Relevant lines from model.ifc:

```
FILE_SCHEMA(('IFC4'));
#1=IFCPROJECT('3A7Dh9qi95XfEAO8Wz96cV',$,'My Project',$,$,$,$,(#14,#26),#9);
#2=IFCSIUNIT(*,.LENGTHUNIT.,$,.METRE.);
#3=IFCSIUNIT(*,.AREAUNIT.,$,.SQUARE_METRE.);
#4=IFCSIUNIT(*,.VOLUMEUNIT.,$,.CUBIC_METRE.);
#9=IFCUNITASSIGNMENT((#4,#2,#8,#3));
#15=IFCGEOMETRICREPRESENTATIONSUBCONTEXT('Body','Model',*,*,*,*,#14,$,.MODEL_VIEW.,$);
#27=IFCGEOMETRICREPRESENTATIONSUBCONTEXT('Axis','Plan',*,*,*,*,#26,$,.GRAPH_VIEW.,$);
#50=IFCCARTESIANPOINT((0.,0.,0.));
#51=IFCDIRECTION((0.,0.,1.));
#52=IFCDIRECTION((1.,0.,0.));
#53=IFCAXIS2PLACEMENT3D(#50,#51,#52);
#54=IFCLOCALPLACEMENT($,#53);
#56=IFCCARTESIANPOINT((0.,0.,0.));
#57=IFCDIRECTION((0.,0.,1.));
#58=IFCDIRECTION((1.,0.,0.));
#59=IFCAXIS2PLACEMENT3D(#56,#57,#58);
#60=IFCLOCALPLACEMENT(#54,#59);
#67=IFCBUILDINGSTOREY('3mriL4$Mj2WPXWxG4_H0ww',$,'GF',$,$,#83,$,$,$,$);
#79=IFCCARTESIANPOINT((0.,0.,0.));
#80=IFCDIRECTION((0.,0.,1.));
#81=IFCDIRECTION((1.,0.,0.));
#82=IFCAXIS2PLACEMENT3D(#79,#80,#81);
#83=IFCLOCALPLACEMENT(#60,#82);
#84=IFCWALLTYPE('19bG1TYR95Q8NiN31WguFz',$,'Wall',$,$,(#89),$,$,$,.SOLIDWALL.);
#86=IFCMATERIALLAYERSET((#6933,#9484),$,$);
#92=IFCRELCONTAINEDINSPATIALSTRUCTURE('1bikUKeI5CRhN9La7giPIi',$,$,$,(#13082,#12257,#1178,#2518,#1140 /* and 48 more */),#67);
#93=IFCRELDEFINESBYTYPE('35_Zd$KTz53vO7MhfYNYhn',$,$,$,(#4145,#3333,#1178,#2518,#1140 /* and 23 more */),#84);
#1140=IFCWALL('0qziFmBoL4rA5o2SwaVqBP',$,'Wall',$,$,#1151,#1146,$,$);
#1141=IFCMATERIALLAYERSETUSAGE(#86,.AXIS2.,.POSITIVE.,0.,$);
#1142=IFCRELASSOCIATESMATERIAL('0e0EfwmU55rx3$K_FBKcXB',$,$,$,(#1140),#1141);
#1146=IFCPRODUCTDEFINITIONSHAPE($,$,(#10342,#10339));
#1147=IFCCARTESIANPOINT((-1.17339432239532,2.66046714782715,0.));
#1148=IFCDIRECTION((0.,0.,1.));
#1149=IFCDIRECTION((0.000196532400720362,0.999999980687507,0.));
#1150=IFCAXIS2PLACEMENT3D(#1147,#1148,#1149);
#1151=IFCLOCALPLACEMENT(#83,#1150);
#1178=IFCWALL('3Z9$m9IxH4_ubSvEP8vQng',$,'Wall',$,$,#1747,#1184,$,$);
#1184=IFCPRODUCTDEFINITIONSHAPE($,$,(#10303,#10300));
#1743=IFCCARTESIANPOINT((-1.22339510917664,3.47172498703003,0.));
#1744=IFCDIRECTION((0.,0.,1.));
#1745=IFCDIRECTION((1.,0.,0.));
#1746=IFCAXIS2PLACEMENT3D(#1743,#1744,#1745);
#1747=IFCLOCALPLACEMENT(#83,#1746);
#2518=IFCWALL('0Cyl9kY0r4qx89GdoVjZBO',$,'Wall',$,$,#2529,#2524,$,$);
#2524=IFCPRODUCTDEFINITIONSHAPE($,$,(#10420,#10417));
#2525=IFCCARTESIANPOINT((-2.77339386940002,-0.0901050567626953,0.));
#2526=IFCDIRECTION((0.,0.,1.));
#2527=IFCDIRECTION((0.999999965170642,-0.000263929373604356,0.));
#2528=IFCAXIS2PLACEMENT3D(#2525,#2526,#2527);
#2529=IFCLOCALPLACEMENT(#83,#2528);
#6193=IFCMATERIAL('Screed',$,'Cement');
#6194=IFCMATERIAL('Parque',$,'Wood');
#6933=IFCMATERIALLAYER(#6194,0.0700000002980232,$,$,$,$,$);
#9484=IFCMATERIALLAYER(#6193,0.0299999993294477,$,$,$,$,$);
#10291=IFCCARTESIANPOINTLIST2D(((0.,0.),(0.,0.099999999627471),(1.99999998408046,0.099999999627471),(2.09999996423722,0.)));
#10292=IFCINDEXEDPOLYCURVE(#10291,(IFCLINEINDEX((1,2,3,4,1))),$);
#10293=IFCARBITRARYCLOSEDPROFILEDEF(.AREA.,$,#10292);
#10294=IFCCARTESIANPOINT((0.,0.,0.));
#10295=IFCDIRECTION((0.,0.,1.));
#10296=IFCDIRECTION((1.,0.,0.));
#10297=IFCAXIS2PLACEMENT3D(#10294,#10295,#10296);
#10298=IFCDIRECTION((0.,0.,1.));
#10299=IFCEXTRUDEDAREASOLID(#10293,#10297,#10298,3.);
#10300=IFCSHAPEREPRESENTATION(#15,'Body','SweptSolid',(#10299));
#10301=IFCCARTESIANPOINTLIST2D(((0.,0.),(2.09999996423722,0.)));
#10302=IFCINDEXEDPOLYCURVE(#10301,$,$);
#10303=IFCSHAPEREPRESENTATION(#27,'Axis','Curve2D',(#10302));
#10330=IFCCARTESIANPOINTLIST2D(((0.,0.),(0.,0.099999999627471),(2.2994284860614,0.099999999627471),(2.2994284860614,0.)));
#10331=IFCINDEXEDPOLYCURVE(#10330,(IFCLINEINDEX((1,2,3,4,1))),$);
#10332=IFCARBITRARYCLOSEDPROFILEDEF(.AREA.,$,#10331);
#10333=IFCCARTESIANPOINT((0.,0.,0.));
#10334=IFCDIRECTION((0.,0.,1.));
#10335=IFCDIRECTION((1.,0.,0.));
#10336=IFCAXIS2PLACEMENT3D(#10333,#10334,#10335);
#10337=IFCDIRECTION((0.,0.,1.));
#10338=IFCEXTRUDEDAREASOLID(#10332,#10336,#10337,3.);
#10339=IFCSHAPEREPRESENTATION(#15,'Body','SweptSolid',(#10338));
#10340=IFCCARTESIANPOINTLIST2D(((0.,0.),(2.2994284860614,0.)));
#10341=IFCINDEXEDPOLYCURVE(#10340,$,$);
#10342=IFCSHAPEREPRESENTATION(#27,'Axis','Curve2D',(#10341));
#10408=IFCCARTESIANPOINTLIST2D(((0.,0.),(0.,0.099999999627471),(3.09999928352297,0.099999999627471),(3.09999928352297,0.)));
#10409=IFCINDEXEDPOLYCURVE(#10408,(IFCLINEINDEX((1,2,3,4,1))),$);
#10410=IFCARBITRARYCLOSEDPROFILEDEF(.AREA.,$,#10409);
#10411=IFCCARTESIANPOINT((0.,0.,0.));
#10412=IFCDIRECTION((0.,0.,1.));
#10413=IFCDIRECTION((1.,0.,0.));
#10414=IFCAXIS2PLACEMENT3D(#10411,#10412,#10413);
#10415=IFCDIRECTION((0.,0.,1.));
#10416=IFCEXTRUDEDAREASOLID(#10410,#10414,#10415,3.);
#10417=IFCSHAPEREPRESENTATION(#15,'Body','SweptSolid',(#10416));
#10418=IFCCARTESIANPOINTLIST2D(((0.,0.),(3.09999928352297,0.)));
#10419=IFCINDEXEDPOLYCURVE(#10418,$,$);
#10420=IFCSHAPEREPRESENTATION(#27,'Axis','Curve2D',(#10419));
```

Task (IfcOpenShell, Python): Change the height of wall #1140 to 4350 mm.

```python
import ifcopenshell
import ifcopenshell.geom
import ifcopenshell.util.representation
import ifcopenshell.util.shape
import ifcopenshell.util.unit

model = ifcopenshell.open("model.ifc")
unit_scale = ifcopenshell.util.unit.calculate_unit_scale(model)
settings = ifcopenshell.geom.settings()


def volume(element):
    """Net volume in cubic metres, openings subtracted."""
    shape = ifcopenshell.geom.create_shape(settings, element)
    return ifcopenshell.util.shape.get_volume(shape.geometry)


wall = model.by_guid("0qziFmBoL4rA5o2SwaVqBP")
before = volume(wall)

body = ifcopenshell.util.representation.get_representation(wall, "Model", "Body")
solid = body.Items[0]
old_height = solid.Depth
solid.Depth = 4.35 / unit_scale
after = volume(wall)

print(f"height {old_height:g} -> {solid.Depth:g}, volume {before:.3f} -> {after:.3f} m3")

model.write("model-out.ifc")
```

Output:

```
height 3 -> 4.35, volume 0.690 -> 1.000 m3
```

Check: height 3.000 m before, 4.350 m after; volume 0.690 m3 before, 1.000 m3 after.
